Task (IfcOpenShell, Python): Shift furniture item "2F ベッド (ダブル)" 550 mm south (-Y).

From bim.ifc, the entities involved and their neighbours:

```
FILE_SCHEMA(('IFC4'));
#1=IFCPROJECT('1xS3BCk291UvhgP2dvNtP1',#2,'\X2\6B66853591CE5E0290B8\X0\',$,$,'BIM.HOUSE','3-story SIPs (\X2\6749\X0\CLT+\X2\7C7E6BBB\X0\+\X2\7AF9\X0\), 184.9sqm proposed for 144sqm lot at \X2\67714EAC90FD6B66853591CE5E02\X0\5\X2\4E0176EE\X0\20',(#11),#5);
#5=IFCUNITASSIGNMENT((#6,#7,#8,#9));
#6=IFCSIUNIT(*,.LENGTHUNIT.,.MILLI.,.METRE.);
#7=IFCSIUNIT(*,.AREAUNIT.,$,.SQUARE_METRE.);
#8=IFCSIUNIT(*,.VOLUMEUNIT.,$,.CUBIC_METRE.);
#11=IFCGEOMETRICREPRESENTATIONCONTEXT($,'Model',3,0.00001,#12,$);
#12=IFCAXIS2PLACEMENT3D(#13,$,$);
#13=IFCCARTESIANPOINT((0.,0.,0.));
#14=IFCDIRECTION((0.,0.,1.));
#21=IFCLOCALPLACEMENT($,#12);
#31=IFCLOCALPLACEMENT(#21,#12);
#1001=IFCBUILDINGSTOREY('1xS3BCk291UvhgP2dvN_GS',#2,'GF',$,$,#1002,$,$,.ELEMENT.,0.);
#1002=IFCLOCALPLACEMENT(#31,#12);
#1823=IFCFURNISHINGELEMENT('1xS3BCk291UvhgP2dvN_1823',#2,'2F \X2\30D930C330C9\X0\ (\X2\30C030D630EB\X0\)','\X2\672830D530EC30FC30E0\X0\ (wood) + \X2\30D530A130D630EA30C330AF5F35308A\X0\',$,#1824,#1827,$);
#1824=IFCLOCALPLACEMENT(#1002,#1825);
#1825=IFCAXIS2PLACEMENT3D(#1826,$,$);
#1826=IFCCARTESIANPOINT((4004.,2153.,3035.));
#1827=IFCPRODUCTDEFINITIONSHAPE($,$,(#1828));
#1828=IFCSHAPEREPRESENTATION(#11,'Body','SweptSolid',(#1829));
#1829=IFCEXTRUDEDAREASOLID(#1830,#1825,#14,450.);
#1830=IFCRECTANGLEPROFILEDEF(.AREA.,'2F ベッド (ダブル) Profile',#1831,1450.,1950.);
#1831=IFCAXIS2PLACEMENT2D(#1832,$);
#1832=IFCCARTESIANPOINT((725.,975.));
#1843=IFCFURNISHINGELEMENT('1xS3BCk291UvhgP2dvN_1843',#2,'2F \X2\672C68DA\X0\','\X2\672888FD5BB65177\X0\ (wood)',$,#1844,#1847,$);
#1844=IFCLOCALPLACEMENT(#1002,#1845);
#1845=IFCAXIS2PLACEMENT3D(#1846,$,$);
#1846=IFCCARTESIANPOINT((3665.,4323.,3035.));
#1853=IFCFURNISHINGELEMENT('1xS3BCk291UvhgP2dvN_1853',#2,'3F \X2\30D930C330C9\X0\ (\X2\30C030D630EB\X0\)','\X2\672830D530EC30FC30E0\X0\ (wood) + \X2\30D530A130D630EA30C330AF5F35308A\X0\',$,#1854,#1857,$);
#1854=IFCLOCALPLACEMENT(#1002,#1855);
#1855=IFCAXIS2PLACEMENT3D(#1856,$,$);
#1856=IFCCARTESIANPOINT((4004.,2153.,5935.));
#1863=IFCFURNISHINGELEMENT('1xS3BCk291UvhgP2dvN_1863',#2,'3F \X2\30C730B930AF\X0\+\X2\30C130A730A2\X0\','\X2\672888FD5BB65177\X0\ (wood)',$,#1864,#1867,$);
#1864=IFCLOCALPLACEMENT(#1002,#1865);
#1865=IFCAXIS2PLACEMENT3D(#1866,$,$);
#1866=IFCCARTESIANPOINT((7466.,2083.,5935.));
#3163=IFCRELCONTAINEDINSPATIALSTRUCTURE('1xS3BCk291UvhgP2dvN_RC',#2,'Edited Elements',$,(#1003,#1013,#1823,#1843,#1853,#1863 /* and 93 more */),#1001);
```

```python
import ifcopenshell
import ifcopenshell.api.geometry
import ifcopenshell.util.placement

model = ifcopenshell.open("bim.ifc")

item = model.by_guid("1xS3BCk291UvhgP2dvN_1823")
matrix = ifcopenshell.util.placement.get_local_placement(item.ObjectPlacement)
matrix[1, 3] -= 550.0
ifcopenshell.api.geometry.edit_object_placement(model, product=item, matrix=matrix, is_si=False)

print(ifcopenshell.util.placement.get_local_placement(item.ObjectPlacement).round(3) + 0.0)

model.write("bim_updated.ifc")
```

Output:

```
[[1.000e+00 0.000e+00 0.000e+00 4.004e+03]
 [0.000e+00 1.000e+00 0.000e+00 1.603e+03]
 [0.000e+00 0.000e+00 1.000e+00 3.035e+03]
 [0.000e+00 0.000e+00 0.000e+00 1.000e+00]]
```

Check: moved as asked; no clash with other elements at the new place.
